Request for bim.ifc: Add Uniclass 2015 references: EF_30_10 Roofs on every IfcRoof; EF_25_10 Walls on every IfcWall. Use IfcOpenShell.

First a look at what the model holds.

```python
import ifcopenshell

model = ifcopenshell.open("bim.ifc")
print(model.schema)
print("classifications:", [c.Name for c in model.by_type("IfcClassification")])
for ifc_class in ("IfcDoor", "IfcRoof", "IfcStair", "IfcWall", "IfcWindow"):
    print(ifc_class, len(model.by_type(ifc_class)))
```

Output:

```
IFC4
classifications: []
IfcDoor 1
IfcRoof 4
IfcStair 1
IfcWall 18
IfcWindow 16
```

```python
import ifcopenshell
import ifcopenshell.api.classification

model = ifcopenshell.open("bim.ifc")

system = ifcopenshell.api.classification.add_classification(model, classification="Uniclass 2015")

codes = {
    "IfcRoof": ("EF_30_10", "Roofs"),
    "IfcWall": ("EF_25_10", "Walls"),
}
for ifc_class, (code, name) in codes.items():
    products = model.by_type(ifc_class)
    ifcopenshell.api.classification.add_reference(
        model, products=products, classification=system, identification=code, name=name
    )
    print(code, len(products))

model.write("bim_v2.ifc")
```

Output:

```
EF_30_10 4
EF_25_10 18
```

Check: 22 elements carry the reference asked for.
